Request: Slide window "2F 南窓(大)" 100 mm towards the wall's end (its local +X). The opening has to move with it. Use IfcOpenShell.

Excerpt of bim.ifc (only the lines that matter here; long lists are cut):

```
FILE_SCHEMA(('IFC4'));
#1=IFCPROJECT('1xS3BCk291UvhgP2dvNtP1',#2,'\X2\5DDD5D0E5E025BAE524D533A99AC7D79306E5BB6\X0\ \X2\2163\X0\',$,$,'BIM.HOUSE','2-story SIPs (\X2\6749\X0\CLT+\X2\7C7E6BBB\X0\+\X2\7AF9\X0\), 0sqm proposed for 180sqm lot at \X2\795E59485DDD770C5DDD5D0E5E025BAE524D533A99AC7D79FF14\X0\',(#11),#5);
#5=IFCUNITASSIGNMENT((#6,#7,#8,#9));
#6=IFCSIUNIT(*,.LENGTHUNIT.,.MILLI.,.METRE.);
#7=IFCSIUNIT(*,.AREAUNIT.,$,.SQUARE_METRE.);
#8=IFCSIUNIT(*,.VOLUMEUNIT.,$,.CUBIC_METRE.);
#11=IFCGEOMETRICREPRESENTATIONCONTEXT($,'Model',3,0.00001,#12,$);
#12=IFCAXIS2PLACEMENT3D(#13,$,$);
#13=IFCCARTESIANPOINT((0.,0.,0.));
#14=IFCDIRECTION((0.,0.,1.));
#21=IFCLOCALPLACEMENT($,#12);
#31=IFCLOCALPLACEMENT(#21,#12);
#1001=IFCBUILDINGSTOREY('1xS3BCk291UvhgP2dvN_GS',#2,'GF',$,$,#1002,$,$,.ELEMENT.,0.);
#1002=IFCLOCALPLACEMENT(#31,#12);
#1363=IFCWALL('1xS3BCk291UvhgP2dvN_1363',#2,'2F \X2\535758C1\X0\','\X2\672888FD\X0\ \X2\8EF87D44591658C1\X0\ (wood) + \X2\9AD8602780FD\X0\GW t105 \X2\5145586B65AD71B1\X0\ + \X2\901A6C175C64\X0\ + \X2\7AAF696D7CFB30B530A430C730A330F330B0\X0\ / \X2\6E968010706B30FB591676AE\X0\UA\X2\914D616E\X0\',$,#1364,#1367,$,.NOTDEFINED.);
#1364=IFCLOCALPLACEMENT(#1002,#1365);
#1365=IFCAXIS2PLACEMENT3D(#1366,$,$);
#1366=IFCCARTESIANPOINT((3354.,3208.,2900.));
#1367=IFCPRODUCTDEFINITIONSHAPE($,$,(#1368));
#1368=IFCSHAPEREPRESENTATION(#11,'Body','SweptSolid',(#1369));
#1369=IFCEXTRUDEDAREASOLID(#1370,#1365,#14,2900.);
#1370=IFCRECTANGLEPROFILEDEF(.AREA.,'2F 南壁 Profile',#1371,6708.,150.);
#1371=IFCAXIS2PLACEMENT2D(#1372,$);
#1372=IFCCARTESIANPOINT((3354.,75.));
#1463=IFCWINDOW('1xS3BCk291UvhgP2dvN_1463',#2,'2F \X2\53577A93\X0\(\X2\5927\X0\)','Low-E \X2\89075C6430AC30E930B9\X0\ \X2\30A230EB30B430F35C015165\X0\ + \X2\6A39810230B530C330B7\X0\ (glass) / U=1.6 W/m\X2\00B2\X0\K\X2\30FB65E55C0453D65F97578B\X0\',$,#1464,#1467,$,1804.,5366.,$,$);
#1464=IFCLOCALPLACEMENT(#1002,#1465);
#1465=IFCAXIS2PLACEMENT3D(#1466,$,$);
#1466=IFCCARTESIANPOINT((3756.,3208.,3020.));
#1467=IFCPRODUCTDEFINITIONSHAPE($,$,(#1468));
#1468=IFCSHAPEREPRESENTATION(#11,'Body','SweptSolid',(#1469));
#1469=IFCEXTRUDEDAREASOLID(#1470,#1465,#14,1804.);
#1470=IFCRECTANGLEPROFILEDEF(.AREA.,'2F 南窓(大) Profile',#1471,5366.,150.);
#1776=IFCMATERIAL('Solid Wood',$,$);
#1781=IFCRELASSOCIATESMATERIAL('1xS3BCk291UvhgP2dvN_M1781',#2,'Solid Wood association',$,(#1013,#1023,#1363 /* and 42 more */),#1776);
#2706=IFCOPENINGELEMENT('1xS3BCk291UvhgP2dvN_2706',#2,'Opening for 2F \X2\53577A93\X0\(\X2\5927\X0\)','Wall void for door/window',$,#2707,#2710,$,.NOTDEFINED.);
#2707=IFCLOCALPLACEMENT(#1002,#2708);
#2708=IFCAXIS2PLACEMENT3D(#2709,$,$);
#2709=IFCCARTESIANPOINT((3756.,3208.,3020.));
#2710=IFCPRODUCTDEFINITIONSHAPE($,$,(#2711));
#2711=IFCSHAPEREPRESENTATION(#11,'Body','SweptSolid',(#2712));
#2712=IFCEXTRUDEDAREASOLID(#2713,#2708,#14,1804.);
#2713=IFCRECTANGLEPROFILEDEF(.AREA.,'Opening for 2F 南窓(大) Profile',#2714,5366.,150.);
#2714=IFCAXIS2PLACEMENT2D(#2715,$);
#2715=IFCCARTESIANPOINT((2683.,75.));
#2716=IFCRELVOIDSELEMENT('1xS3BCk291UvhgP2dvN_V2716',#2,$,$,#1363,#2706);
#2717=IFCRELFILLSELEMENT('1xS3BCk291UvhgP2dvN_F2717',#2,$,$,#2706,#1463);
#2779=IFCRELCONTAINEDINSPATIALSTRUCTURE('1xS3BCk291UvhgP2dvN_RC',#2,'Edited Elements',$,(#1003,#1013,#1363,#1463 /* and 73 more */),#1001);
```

```python
import ifcopenshell
import ifcopenshell.api.geometry
import ifcopenshell.util.placement
import ifcopenshell.util.unit

model = ifcopenshell.open("bim.ifc")
unit_scale = ifcopenshell.util.unit.calculate_unit_scale(model)

window = model.by_guid("1xS3BCk291UvhgP2dvN_1463")
opening = window.FillsVoids[0].RelatingOpeningElement
wall = opening.VoidsElements[0].RelatingBuildingElement

wall_matrix = ifcopenshell.util.placement.get_local_placement(wall.ObjectPlacement)
shift = wall_matrix[:3, 0] * 0.1 / unit_scale
before = ifcopenshell.util.placement.get_local_placement(window.ObjectPlacement)[:3, 3].copy()

# The window is not placed relative to its opening, so move both.
for product in (opening, window):
    matrix = ifcopenshell.util.placement.get_local_placement(product.ObjectPlacement)
    matrix[:3, 3] += shift
    ifcopenshell.api.geometry.edit_object_placement(model, product=product, matrix=matrix, is_si=False)

after = ifcopenshell.util.placement.get_local_placement(window.ObjectPlacement)[:3, 3]
print("window moved by", (after - before).round(3) + 0.0)

model.write("bim_updated.ifc")
```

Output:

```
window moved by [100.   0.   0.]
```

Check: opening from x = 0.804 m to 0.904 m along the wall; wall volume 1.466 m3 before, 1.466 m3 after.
